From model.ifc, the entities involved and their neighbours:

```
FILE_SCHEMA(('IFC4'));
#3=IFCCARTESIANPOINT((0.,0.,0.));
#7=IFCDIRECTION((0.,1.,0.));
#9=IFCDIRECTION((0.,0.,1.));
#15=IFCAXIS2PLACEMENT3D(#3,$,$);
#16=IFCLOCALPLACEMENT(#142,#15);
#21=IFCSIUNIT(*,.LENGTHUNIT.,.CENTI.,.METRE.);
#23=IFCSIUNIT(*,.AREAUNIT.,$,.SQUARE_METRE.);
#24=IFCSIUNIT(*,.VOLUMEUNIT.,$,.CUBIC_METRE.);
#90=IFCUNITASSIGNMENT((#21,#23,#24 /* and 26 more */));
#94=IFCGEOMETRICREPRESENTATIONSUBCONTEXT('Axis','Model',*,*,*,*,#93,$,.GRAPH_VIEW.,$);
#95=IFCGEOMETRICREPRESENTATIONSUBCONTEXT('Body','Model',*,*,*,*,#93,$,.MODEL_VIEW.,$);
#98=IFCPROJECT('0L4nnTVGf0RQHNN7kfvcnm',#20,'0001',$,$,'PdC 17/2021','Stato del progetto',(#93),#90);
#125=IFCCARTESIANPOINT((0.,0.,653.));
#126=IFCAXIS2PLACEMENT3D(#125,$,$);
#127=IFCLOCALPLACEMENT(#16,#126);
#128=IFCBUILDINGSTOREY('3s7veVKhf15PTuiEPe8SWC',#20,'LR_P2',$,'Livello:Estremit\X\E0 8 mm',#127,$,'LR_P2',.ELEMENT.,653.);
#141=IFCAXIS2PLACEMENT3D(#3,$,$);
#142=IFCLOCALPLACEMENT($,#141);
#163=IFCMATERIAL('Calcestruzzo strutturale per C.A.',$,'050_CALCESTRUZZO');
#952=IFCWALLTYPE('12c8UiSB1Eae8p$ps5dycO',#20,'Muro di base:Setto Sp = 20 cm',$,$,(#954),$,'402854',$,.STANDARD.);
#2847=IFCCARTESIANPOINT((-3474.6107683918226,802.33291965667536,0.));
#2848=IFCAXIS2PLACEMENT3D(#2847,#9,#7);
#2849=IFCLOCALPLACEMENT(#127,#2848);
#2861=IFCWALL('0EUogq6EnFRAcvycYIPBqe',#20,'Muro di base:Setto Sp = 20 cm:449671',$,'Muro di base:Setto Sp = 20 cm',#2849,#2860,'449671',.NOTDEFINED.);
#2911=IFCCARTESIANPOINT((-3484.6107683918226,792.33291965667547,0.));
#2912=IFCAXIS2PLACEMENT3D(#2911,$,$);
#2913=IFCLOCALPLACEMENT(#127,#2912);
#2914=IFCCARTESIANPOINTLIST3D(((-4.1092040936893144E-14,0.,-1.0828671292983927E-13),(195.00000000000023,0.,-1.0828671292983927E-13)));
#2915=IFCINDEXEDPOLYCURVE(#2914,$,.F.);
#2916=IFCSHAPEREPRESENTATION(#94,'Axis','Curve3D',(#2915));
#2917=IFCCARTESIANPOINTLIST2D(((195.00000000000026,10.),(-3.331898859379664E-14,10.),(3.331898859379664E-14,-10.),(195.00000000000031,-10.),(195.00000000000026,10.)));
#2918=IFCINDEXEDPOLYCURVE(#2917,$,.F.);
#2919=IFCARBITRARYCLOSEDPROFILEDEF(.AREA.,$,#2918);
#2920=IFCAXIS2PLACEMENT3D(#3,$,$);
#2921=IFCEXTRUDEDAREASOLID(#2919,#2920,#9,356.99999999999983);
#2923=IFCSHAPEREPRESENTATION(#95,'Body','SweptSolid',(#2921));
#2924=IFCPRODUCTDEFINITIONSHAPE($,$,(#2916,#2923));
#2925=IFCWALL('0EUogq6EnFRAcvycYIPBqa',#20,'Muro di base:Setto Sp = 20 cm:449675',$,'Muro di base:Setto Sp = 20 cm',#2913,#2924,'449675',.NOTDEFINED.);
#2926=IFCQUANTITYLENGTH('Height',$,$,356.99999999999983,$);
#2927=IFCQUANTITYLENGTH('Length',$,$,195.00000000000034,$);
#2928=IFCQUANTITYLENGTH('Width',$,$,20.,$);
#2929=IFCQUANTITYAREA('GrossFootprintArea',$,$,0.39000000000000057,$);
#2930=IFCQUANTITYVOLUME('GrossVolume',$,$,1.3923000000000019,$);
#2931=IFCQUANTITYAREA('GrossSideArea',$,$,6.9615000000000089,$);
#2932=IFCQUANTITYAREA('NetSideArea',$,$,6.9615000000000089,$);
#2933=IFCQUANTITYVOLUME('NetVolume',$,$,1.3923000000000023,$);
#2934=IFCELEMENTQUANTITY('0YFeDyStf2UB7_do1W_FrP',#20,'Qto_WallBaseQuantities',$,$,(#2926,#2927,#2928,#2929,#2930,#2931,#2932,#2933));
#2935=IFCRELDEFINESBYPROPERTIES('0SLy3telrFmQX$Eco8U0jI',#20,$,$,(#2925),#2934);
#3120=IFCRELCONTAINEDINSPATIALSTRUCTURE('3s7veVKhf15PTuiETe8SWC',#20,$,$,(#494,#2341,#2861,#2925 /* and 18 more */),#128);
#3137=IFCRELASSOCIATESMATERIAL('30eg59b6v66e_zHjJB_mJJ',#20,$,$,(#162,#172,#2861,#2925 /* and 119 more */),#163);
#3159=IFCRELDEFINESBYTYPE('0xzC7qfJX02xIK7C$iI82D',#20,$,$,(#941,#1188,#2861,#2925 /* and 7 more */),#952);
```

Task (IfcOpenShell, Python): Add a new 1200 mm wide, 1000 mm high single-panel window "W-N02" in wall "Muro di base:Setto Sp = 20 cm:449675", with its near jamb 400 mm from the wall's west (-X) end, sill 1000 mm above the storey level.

```python
import numpy as np
import ifcopenshell
import ifcopenshell.api.feature
import ifcopenshell.api.geometry
import ifcopenshell.api.pset
import ifcopenshell.api.root
import ifcopenshell.api.spatial
import ifcopenshell.geom
import ifcopenshell.util.element
import ifcopenshell.util.placement
import ifcopenshell.util.representation
import ifcopenshell.util.shape
import ifcopenshell.util.unit

model = ifcopenshell.open("model.ifc")
unit_scale = ifcopenshell.util.unit.calculate_unit_scale(model)
area_scale = ifcopenshell.util.unit.calculate_unit_scale(model, "AREAUNIT")
volume_scale = ifcopenshell.util.unit.calculate_unit_scale(model, "VOLUMEUNIT")
settings = ifcopenshell.geom.settings()


def volume(element):
    """Net volume in cubic metres, openings subtracted."""
    shape = ifcopenshell.geom.create_shape(settings, element)
    return ifcopenshell.util.shape.get_volume(shape.geometry)


wall = model.by_guid("0EUogq6EnFRAcvycYIPBqa")
storey = ifcopenshell.util.element.get_container(wall, ifc_class="IfcBuildingStorey")
context = ifcopenshell.util.representation.get_context(model, "Model", "Body", "MODEL_VIEW")
before = volume(wall)

width, height, from_end, sill = 1.2, 1, 0.4, 1  # metres

# The wall runs along its own X axis, and the end named is its -X end.
wall_shape = ifcopenshell.geom.create_shape(settings, wall)
x, y, z = ifcopenshell.util.shape.get_vertices(wall_shape.geometry).T
start = x.min() + from_end
face, thickness = float(y.min()), float(y.max() - y.min())
wall_matrix = ifcopenshell.util.placement.get_local_placement(wall.ObjectPlacement)
level = ifcopenshell.util.placement.get_local_placement(storey.ObjectPlacement)[2, 3]


def in_wall(x, y):
    """Placement at x, y metres in the wall's axes, at sill height."""
    matrix = wall_matrix.copy()
    matrix[:, 3] = wall_matrix @ np.array([x / unit_scale, y / unit_scale, 0.0, 1.0])
    matrix[2, 3] = level + sill / unit_scale
    return matrix


# Opening: a box that overshoots both wall faces by 50 mm.
opening = ifcopenshell.api.root.create_entity(model, ifc_class="IfcOpeningElement", predefined_type="OPENING")
box = ifcopenshell.api.geometry.add_wall_representation(
    model, context=context, length=width, height=height, thickness=thickness + 0.1
)
ifcopenshell.api.geometry.assign_representation(model, product=opening, representation=box)
ifcopenshell.api.geometry.edit_object_placement(model, product=opening, matrix=in_wall(start, face - 0.05), is_si=False)
ifcopenshell.api.feature.add_feature(model, feature=opening, element=wall)

window = ifcopenshell.api.root.create_entity(model, ifc_class="IfcWindow", name="W-N02", predefined_type="WINDOW")
window.OverallWidth, window.OverallHeight = width / unit_scale, height / unit_scale
window.PartitioningType = "SINGLE_PANEL"
body = ifcopenshell.api.geometry.add_window_representation(
    model,
    context=context,
    overall_width=window.OverallWidth,
    overall_height=window.OverallHeight,
    partition_type="SINGLE_PANEL",
)
ifcopenshell.api.geometry.assign_representation(model, product=window, representation=body)
ifcopenshell.api.spatial.assign_container(model, products=[window], relating_structure=storey)
ifcopenshell.api.feature.add_filling(model, opening=opening, element=window)

# Centre the window in the wall's thickness.
ifcopenshell.api.geometry.edit_object_placement(model, product=window, matrix=in_wall(start, face), is_si=False)
window_shape = ifcopenshell.geom.create_shape(settings, window)
depth = ifcopenshell.util.shape.get_vertices(window_shape.geometry)[:, 1]
offset = face + thickness / 2 - (depth.min() + depth.max()) / 2
ifcopenshell.api.geometry.edit_object_placement(model, product=window, matrix=in_wall(start, offset), is_si=False)

after = volume(wall)

# Update the wall's stored quantities.
qto = model.by_id(ifcopenshell.util.element.get_pset(wall, "Qto_WallBaseQuantities", should_inherit=False)["id"])
ifcopenshell.api.pset.edit_qto(model, qto=qto, properties={
    "NetSideArea": after / thickness / area_scale,
    "NetVolume": after / volume_scale,
})

print(f"wall volume {before:.3f} -> {after:.3f} m3")

model.write("model-out.ifc")
```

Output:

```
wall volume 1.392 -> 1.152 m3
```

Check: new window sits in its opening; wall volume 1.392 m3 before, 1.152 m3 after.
